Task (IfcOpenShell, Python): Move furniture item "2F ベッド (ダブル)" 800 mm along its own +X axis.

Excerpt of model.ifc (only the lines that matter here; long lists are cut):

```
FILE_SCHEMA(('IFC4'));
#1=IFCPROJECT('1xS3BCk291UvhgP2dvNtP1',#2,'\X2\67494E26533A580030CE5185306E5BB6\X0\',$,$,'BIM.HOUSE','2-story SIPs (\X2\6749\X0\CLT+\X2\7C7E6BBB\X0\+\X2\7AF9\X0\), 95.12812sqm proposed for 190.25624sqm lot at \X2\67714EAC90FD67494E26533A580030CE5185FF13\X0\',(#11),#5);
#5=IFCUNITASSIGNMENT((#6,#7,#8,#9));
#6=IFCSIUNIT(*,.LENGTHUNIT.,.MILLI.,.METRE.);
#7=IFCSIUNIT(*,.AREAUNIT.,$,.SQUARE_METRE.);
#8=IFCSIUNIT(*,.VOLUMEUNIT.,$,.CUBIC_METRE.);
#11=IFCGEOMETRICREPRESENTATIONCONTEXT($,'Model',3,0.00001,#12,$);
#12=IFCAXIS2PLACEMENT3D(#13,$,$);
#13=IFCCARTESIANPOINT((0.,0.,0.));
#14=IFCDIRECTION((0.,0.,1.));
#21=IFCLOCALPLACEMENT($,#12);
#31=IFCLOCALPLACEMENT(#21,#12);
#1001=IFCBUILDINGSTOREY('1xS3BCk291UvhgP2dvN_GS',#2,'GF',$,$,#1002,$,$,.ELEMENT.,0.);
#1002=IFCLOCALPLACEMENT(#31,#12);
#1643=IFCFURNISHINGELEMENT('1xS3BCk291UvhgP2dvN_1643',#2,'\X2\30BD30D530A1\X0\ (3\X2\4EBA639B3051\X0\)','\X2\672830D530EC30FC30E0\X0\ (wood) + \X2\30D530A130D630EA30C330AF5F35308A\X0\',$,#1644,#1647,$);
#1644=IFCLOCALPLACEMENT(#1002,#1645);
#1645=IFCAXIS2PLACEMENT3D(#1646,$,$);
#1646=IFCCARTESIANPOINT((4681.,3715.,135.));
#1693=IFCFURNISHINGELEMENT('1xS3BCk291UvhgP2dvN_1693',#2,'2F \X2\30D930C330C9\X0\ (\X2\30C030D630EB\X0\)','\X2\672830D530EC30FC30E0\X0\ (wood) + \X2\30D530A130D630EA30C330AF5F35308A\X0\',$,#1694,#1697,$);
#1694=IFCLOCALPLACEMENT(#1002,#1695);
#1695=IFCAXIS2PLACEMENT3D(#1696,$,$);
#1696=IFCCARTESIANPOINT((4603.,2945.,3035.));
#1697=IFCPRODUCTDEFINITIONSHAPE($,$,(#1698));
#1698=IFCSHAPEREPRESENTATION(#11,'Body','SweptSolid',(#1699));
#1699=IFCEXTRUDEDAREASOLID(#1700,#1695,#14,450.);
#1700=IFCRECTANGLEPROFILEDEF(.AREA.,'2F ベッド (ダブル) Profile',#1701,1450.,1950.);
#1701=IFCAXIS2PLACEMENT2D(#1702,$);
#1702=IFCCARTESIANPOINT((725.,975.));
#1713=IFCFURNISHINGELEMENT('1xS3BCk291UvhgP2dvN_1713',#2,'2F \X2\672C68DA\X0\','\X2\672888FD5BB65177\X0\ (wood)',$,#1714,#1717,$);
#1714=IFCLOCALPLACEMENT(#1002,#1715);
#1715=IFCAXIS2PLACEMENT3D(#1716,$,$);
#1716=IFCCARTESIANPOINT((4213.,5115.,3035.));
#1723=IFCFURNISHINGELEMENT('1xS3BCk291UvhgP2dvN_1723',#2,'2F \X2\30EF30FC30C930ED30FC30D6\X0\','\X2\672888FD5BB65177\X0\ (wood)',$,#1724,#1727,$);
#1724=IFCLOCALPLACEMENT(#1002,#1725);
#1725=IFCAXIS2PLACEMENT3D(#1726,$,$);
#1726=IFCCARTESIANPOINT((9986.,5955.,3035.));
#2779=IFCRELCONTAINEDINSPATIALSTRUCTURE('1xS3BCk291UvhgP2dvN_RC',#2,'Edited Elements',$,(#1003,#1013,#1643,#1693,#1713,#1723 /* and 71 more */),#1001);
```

```python
import ifcopenshell
import ifcopenshell.api.geometry
import ifcopenshell.util.placement

model = ifcopenshell.open("model.ifc")

item = model.by_id(1693)
matrix = ifcopenshell.util.placement.get_local_placement(item.ObjectPlacement)
matrix[:3, 3] += matrix[:3, 0] * 800.0
ifcopenshell.api.geometry.edit_object_placement(model, product=item, matrix=matrix, is_si=False)

print(ifcopenshell.util.placement.get_local_placement(item.ObjectPlacement).round(3) + 0.0)

model.write("model-out.ifc")
```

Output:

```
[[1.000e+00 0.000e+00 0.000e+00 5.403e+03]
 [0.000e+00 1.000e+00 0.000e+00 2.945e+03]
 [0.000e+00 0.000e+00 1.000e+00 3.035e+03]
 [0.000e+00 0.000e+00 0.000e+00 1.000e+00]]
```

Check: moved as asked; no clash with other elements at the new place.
